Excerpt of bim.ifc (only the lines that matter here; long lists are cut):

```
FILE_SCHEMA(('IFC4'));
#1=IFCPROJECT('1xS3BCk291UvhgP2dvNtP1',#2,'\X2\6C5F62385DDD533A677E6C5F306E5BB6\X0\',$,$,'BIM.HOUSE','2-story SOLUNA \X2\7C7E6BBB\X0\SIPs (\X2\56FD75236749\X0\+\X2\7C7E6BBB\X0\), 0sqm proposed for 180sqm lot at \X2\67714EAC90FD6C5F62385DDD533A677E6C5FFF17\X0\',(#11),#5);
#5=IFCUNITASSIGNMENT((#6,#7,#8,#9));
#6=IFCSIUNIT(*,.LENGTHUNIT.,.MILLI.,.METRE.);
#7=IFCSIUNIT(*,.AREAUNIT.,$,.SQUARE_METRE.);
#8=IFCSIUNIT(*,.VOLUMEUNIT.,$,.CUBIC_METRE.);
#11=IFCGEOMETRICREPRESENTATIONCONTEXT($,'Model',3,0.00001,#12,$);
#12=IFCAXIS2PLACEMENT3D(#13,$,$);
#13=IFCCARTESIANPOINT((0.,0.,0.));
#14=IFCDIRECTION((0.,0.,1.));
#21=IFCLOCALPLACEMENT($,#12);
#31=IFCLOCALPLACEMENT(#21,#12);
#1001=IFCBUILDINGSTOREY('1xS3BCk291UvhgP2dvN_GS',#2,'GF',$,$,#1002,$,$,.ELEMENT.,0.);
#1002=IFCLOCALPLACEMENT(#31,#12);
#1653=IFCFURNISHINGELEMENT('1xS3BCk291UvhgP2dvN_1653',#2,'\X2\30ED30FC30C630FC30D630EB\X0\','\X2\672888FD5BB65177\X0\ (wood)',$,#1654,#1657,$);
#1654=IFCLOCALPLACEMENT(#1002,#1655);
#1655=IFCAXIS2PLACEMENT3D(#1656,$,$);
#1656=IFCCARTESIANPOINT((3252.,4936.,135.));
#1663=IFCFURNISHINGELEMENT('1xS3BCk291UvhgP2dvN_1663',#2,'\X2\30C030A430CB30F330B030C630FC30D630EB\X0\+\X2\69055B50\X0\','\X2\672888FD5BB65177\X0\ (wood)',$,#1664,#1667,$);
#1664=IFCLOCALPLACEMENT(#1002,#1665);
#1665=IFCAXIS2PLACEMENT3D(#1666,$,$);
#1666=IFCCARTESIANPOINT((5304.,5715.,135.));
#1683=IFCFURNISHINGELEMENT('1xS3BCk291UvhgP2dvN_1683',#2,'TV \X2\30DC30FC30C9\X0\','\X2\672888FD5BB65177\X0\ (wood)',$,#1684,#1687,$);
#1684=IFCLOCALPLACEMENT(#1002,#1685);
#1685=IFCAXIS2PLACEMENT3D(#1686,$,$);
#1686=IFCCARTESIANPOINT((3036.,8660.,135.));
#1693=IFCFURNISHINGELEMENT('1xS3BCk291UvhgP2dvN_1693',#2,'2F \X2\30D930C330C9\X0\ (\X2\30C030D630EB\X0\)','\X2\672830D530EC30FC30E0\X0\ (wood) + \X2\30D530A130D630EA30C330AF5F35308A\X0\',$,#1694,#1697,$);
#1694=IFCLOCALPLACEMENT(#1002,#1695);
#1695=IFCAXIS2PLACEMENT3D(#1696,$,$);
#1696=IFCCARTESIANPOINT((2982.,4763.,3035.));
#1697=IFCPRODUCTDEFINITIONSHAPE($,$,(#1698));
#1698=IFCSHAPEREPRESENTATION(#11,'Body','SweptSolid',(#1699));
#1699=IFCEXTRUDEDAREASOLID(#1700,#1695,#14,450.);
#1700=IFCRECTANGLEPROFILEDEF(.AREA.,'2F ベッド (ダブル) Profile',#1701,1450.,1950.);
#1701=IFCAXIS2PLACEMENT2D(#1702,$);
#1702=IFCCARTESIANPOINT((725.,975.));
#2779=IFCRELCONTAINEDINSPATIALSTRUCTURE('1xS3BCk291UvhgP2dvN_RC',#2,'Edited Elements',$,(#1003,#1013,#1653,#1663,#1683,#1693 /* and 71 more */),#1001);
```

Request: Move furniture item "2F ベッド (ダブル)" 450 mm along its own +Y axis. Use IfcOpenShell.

```python
import ifcopenshell
import ifcopenshell.api.geometry
import ifcopenshell.util.placement
import ifcopenshell.util.unit

model = ifcopenshell.open("bim.ifc")
unit_scale = ifcopenshell.util.unit.calculate_unit_scale(model)

item = model.by_guid("1xS3BCk291UvhgP2dvN_1693")
matrix = ifcopenshell.util.placement.get_local_placement(item.ObjectPlacement)
matrix[:3, 3] += matrix[:3, 1] * 0.45 / unit_scale
ifcopenshell.api.geometry.edit_object_placement(model, product=item, matrix=matrix, is_si=False)

print(ifcopenshell.util.placement.get_local_placement(item.ObjectPlacement).round(3) + 0.0)

model.write("bim_v2.ifc")
```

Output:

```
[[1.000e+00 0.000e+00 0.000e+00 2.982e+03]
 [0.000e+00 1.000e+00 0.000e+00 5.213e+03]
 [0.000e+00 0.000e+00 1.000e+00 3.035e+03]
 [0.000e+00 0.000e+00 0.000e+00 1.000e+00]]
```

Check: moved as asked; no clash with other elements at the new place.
